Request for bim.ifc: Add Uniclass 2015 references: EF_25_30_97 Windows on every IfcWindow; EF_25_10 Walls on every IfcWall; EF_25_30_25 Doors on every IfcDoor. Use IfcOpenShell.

First a look at what the model holds.

```python
import ifcopenshell

model = ifcopenshell.open("bim.ifc")
print(model.schema)
print("classifications:", [c.Name for c in model.by_type("IfcClassification")])
for ifc_class in ("IfcDoor", "IfcRoof", "IfcStair", "IfcWall", "IfcWindow"):
    print(ifc_class, len(model.by_type(ifc_class)))
```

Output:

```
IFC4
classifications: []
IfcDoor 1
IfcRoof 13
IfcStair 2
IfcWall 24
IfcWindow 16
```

```python
import ifcopenshell
import ifcopenshell.api.classification

model = ifcopenshell.open("bim.ifc")

system = ifcopenshell.api.classification.add_classification(model, classification="Uniclass 2015")

codes = {
    "IfcWindow": ("EF_25_30_97", "Windows"),
    "IfcWall": ("EF_25_10", "Walls"),
    "IfcDoor": ("EF_25_30_25", "Doors"),
}
for ifc_class, (code, name) in codes.items():
    products = model.by_type(ifc_class)
    ifcopenshell.api.classification.add_reference(
        model, products=products, classification=system, identification=code, name=name
    )
    print(code, len(products))

model.write("bim_edited.ifc")
```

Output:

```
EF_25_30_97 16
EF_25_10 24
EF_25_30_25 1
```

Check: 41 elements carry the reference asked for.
